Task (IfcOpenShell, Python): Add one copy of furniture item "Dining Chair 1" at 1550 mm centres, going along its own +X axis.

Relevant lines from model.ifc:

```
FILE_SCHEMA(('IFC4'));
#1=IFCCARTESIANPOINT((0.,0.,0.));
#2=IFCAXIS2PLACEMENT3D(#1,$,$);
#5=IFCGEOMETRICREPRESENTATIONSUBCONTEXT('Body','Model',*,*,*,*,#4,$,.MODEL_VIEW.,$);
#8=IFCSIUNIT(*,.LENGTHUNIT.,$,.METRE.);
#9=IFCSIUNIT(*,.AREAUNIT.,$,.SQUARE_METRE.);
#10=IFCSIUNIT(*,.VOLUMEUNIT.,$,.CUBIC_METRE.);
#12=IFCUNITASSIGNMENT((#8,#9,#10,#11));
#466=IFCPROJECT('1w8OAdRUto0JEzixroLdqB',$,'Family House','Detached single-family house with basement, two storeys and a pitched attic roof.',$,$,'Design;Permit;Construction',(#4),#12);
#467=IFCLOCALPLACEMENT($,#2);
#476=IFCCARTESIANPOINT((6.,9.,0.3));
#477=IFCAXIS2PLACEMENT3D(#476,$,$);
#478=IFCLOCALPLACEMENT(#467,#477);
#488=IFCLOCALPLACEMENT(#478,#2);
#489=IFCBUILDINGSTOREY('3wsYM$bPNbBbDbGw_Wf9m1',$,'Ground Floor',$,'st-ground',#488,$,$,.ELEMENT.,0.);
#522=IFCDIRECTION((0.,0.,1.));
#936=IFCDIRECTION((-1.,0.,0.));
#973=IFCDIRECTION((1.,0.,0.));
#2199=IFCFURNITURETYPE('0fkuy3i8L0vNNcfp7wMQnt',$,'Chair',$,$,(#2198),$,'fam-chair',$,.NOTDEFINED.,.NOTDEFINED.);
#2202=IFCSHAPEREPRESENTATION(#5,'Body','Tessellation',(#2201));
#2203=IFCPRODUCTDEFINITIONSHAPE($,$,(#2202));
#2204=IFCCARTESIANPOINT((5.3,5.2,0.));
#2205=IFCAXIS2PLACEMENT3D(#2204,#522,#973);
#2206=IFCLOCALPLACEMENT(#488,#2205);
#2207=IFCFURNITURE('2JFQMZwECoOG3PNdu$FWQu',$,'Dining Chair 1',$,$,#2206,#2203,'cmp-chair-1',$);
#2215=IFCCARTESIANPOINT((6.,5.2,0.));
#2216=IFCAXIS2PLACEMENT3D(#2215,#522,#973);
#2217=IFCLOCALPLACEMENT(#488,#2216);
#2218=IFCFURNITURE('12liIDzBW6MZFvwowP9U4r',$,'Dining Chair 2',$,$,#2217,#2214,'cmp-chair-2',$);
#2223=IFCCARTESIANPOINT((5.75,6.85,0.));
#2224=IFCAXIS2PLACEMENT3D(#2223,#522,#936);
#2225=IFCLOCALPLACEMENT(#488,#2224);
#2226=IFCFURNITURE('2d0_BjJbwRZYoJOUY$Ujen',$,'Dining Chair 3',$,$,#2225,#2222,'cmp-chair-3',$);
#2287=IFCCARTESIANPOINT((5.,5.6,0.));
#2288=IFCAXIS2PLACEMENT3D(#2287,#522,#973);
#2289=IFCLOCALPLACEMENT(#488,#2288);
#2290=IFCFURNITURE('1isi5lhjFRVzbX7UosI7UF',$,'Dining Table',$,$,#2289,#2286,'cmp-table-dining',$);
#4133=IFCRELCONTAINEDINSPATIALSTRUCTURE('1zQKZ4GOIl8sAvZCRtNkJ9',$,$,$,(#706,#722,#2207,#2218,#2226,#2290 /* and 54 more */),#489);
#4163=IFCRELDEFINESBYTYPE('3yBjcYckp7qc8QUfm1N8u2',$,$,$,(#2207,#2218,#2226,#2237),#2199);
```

```python
import ifcopenshell
import ifcopenshell.api.geometry
import ifcopenshell.api.root
import ifcopenshell.util.element
import ifcopenshell.util.placement

model = ifcopenshell.open("model.ifc")

source = model.by_guid("2JFQMZwECoOG3PNdu$FWQu")
base = ifcopenshell.util.placement.get_local_placement(source.ObjectPlacement)
step = base[:3, 0] * 1.55

for i in range(1, 2):
    copy = ifcopenshell.api.root.copy_class(model, product=source)
    copy.Representation = ifcopenshell.util.element.copy_deep(
        model, source.Representation, exclude=["IfcGeometricRepresentationContext", "IfcRepresentationMap"]
    )
    copy.Tag = None
    matrix = base.copy()
    matrix[:3, 3] += i * step
    print("added at", matrix[:3, 3].round(3) + 0.0)
    ifcopenshell.api.geometry.edit_object_placement(model, product=copy, matrix=matrix, is_si=False)

model.write("model_rev.ifc")
```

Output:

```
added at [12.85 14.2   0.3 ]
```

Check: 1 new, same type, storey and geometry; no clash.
